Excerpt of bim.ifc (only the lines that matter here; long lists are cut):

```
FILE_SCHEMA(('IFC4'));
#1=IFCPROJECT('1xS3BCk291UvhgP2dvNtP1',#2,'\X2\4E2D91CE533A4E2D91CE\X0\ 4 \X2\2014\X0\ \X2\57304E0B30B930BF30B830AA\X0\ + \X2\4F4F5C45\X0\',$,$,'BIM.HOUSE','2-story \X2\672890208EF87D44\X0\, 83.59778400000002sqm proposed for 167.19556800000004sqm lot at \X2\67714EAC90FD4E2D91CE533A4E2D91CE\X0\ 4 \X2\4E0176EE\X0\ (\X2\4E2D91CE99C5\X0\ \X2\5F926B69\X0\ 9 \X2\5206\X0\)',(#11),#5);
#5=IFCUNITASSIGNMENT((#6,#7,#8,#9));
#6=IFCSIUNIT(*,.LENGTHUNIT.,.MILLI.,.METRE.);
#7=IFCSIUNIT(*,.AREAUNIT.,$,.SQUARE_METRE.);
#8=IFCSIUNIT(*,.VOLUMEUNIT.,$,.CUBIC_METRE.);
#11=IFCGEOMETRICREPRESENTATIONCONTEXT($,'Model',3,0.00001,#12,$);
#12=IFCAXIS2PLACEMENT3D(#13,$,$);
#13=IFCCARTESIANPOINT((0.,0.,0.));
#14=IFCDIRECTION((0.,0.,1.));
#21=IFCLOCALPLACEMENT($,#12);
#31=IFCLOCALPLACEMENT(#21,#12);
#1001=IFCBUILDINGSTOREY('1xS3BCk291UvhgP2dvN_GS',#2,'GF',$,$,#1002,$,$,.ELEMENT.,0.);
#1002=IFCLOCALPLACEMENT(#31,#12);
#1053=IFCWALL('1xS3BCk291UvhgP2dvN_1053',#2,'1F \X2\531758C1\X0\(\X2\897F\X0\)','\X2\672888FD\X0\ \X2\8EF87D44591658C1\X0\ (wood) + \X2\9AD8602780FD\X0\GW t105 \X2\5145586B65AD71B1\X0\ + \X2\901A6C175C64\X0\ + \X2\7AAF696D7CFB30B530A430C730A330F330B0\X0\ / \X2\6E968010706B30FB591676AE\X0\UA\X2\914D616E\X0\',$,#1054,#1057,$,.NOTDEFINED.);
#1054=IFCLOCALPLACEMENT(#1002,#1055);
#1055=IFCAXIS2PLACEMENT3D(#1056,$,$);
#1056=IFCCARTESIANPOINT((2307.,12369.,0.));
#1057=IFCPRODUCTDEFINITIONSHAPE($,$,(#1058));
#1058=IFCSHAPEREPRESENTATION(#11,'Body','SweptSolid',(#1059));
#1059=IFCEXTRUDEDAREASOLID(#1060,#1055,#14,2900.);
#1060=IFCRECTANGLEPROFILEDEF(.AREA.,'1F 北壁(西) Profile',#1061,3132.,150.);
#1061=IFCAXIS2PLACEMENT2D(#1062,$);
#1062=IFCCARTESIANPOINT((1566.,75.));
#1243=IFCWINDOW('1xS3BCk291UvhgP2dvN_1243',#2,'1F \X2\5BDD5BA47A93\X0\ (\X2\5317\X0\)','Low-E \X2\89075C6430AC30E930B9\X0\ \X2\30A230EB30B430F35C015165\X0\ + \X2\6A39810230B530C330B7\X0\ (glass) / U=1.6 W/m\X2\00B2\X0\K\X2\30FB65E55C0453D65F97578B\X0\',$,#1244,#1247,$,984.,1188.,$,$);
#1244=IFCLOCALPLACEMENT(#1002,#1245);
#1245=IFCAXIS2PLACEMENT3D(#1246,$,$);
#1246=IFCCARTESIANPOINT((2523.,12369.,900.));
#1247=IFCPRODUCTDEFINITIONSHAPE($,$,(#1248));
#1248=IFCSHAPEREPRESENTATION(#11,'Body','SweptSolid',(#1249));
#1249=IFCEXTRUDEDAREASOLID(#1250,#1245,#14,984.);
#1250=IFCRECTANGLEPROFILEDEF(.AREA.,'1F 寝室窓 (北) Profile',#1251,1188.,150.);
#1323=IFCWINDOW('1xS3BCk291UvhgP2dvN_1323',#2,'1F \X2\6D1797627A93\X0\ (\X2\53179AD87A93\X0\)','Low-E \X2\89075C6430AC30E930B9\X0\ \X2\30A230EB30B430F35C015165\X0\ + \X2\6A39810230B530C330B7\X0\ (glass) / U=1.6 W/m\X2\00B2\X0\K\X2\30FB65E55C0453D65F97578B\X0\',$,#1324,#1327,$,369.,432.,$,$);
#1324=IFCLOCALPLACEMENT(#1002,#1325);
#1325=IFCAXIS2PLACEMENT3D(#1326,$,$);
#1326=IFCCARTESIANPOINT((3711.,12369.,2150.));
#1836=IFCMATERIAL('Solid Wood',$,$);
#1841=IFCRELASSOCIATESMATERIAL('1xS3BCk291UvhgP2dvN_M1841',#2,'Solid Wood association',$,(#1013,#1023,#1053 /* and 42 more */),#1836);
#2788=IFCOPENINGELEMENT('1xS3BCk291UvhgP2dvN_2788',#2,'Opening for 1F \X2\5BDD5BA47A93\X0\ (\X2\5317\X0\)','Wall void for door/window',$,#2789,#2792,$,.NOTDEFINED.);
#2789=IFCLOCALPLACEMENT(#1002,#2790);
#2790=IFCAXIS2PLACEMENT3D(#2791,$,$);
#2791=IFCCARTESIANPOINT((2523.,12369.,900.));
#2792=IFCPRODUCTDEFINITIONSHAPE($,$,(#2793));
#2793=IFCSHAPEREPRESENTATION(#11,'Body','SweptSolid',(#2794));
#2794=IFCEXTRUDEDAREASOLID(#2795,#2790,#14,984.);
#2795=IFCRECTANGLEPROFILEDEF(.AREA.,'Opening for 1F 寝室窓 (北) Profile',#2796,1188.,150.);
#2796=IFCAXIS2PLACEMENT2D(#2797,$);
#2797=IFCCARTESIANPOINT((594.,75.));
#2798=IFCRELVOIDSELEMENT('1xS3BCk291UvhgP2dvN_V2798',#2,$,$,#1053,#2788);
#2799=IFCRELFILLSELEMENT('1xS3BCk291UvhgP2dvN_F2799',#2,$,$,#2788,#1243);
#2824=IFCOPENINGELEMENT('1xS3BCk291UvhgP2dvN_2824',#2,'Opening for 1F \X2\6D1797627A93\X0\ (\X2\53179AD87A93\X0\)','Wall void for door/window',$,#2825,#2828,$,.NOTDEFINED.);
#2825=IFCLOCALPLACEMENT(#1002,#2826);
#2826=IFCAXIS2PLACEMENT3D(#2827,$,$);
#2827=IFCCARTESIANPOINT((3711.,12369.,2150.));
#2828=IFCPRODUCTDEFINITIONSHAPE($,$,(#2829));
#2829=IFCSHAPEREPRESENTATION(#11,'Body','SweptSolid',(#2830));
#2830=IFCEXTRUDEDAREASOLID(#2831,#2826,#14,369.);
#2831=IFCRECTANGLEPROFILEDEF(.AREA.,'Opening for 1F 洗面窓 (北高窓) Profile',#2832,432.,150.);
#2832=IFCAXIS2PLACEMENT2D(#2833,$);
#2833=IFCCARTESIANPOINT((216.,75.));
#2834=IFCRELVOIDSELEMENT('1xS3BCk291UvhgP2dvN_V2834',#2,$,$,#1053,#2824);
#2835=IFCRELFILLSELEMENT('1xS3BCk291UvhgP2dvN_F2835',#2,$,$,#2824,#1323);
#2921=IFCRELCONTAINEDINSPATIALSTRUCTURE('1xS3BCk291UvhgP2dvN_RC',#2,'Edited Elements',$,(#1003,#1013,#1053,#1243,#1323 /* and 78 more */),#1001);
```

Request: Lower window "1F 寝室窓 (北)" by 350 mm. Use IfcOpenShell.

```python
import numpy as np
import ifcopenshell
import ifcopenshell.api.geometry
import ifcopenshell.util.placement
import ifcopenshell.util.unit

model = ifcopenshell.open("bim.ifc")
unit_scale = ifcopenshell.util.unit.calculate_unit_scale(model)

window = model.by_id(1243)
opening = window.FillsVoids[0].RelatingOpeningElement
dz = -0.35 / unit_scale

shift = np.array([0.0, 0.0, dz])
# The window is not placed relative to its opening, so move both.
for product in (opening, window):
    matrix = ifcopenshell.util.placement.get_local_placement(product.ObjectPlacement)
    matrix[:3, 3] += shift
    ifcopenshell.api.geometry.edit_object_placement(model, product=product, matrix=matrix, is_si=False)

print(f"moved by {dz * unit_scale:+.3f} m")

model.write("bim_edited.ifc")
```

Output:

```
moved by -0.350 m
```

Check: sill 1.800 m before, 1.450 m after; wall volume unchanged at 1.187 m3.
